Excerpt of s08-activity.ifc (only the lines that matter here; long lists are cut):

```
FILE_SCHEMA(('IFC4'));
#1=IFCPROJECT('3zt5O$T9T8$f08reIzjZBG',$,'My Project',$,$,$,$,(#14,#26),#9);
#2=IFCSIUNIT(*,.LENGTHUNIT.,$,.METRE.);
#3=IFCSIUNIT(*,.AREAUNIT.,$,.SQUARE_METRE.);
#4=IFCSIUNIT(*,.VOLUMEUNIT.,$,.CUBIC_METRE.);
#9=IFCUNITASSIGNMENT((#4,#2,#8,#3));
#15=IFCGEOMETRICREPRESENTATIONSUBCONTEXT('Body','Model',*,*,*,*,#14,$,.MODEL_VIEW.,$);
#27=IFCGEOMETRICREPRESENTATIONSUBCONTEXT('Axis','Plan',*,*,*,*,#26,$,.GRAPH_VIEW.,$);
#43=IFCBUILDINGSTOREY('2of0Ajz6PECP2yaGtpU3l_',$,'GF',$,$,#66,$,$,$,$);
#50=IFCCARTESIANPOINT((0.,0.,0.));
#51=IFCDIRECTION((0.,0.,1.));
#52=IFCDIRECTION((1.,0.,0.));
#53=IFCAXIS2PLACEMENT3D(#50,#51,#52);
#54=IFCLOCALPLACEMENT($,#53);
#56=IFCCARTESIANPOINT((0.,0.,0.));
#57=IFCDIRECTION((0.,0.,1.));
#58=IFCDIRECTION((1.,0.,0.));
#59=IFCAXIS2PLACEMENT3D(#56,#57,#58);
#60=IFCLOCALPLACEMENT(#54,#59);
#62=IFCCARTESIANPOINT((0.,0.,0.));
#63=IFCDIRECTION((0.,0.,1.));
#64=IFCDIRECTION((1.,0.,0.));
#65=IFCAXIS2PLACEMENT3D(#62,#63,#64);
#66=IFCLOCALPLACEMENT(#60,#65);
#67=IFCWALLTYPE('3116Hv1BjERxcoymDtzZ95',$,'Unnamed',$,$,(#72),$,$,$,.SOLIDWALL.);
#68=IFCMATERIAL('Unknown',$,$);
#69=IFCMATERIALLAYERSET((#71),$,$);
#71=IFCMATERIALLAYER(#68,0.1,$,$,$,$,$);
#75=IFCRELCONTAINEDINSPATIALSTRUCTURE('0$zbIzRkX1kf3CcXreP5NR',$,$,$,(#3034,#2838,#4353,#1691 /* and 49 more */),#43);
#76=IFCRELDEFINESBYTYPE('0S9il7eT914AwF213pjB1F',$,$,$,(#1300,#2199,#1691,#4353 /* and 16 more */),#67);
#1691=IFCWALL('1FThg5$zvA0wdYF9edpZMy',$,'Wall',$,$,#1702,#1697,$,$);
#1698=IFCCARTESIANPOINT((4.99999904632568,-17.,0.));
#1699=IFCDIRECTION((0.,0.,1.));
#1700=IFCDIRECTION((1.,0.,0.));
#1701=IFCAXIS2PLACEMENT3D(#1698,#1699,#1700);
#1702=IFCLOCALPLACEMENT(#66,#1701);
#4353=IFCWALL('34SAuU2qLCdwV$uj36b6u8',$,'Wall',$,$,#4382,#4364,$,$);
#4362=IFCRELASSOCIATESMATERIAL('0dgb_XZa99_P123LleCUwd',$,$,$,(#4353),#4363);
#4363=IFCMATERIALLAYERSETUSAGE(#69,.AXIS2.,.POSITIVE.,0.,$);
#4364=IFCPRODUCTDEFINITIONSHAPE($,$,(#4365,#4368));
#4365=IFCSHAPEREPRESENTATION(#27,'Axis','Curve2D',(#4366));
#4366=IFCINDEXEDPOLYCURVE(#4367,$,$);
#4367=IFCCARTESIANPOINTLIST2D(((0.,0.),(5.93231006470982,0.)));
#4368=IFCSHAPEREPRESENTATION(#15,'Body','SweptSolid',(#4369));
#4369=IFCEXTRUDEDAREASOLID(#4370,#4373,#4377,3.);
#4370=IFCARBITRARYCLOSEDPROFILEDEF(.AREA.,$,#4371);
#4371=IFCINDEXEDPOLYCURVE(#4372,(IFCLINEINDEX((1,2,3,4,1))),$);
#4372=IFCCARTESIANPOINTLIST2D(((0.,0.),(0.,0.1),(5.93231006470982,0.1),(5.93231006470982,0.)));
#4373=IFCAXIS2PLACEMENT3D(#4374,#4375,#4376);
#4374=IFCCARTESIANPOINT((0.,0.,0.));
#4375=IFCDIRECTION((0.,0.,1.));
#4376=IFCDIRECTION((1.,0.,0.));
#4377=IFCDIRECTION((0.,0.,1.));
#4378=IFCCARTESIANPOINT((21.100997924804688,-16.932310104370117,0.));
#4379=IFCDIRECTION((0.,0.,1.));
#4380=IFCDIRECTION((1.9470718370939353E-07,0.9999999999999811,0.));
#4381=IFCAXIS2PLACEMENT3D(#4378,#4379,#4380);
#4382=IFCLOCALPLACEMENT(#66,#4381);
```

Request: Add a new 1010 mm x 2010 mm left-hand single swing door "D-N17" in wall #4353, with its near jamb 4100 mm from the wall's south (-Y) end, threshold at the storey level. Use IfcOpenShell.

```python
import numpy as np
import ifcopenshell
import ifcopenshell.api.feature
import ifcopenshell.api.geometry
import ifcopenshell.api.root
import ifcopenshell.api.spatial
import ifcopenshell.geom
import ifcopenshell.util.element
import ifcopenshell.util.placement
import ifcopenshell.util.representation
import ifcopenshell.util.shape
import ifcopenshell.util.unit

model = ifcopenshell.open("s08-activity.ifc")
unit_scale = ifcopenshell.util.unit.calculate_unit_scale(model)
settings = ifcopenshell.geom.settings()


def volume(element):
    """Net volume in cubic metres, openings subtracted."""
    shape = ifcopenshell.geom.create_shape(settings, element)
    return ifcopenshell.util.shape.get_volume(shape.geometry)


wall = model.by_id(4353)
storey = ifcopenshell.util.element.get_container(wall, ifc_class="IfcBuildingStorey")
context = ifcopenshell.util.representation.get_context(model, "Model", "Body", "MODEL_VIEW")
before = volume(wall)

width, height, from_end, sill = 1.01, 2.01, 4.1, 0.0  # metres

# The wall runs along its own X axis, and the end named is its -X end.
wall_shape = ifcopenshell.geom.create_shape(settings, wall)
x, y, z = ifcopenshell.util.shape.get_vertices(wall_shape.geometry).T
start = x.min() + from_end
face, thickness = float(y.min()), float(y.max() - y.min())
wall_matrix = ifcopenshell.util.placement.get_local_placement(wall.ObjectPlacement)
level = ifcopenshell.util.placement.get_local_placement(storey.ObjectPlacement)[2, 3]


def in_wall(x, y):
    """Placement at x, y metres in the wall's axes, at sill height."""
    matrix = wall_matrix.copy()
    matrix[:, 3] = wall_matrix @ np.array([x / unit_scale, y / unit_scale, 0.0, 1.0])
    matrix[2, 3] = level + sill / unit_scale
    return matrix


# Opening: a box that overshoots both wall faces by 50 mm.
opening = ifcopenshell.api.root.create_entity(model, ifc_class="IfcOpeningElement", predefined_type="OPENING")
box = ifcopenshell.api.geometry.add_wall_representation(
    model, context=context, length=width, height=height, thickness=thickness + 0.1
)
ifcopenshell.api.geometry.assign_representation(model, product=opening, representation=box)
ifcopenshell.api.geometry.edit_object_placement(model, product=opening, matrix=in_wall(start, face - 0.05), is_si=False)
ifcopenshell.api.feature.add_feature(model, feature=opening, element=wall)

door = ifcopenshell.api.root.create_entity(model, ifc_class="IfcDoor", name="D-N17", predefined_type="DOOR")
door.OverallWidth, door.OverallHeight = width / unit_scale, height / unit_scale
door.OperationType = "SINGLE_SWING_LEFT"
body = ifcopenshell.api.geometry.add_door_representation(
    model,
    context=context,
    overall_width=door.OverallWidth,
    overall_height=door.OverallHeight,
    operation_type="SINGLE_SWING_LEFT",
    lining_properties={"LiningDepth": thickness / unit_scale, "ThresholdDepth": thickness / unit_scale},
)
ifcopenshell.api.geometry.assign_representation(model, product=door, representation=body)
ifcopenshell.api.spatial.assign_container(model, products=[door], relating_structure=storey)
ifcopenshell.api.feature.add_filling(model, opening=opening, element=door)

# The lining spans the wall, so the door starts at the wall face.
ifcopenshell.api.geometry.edit_object_placement(model, product=door, matrix=in_wall(start, face), is_si=False)

after = volume(wall)

print(f"wall volume {before:.3f} -> {after:.3f} m3")

model.write("s08-activity-out.ifc")
```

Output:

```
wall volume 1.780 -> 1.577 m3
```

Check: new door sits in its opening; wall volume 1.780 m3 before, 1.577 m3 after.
